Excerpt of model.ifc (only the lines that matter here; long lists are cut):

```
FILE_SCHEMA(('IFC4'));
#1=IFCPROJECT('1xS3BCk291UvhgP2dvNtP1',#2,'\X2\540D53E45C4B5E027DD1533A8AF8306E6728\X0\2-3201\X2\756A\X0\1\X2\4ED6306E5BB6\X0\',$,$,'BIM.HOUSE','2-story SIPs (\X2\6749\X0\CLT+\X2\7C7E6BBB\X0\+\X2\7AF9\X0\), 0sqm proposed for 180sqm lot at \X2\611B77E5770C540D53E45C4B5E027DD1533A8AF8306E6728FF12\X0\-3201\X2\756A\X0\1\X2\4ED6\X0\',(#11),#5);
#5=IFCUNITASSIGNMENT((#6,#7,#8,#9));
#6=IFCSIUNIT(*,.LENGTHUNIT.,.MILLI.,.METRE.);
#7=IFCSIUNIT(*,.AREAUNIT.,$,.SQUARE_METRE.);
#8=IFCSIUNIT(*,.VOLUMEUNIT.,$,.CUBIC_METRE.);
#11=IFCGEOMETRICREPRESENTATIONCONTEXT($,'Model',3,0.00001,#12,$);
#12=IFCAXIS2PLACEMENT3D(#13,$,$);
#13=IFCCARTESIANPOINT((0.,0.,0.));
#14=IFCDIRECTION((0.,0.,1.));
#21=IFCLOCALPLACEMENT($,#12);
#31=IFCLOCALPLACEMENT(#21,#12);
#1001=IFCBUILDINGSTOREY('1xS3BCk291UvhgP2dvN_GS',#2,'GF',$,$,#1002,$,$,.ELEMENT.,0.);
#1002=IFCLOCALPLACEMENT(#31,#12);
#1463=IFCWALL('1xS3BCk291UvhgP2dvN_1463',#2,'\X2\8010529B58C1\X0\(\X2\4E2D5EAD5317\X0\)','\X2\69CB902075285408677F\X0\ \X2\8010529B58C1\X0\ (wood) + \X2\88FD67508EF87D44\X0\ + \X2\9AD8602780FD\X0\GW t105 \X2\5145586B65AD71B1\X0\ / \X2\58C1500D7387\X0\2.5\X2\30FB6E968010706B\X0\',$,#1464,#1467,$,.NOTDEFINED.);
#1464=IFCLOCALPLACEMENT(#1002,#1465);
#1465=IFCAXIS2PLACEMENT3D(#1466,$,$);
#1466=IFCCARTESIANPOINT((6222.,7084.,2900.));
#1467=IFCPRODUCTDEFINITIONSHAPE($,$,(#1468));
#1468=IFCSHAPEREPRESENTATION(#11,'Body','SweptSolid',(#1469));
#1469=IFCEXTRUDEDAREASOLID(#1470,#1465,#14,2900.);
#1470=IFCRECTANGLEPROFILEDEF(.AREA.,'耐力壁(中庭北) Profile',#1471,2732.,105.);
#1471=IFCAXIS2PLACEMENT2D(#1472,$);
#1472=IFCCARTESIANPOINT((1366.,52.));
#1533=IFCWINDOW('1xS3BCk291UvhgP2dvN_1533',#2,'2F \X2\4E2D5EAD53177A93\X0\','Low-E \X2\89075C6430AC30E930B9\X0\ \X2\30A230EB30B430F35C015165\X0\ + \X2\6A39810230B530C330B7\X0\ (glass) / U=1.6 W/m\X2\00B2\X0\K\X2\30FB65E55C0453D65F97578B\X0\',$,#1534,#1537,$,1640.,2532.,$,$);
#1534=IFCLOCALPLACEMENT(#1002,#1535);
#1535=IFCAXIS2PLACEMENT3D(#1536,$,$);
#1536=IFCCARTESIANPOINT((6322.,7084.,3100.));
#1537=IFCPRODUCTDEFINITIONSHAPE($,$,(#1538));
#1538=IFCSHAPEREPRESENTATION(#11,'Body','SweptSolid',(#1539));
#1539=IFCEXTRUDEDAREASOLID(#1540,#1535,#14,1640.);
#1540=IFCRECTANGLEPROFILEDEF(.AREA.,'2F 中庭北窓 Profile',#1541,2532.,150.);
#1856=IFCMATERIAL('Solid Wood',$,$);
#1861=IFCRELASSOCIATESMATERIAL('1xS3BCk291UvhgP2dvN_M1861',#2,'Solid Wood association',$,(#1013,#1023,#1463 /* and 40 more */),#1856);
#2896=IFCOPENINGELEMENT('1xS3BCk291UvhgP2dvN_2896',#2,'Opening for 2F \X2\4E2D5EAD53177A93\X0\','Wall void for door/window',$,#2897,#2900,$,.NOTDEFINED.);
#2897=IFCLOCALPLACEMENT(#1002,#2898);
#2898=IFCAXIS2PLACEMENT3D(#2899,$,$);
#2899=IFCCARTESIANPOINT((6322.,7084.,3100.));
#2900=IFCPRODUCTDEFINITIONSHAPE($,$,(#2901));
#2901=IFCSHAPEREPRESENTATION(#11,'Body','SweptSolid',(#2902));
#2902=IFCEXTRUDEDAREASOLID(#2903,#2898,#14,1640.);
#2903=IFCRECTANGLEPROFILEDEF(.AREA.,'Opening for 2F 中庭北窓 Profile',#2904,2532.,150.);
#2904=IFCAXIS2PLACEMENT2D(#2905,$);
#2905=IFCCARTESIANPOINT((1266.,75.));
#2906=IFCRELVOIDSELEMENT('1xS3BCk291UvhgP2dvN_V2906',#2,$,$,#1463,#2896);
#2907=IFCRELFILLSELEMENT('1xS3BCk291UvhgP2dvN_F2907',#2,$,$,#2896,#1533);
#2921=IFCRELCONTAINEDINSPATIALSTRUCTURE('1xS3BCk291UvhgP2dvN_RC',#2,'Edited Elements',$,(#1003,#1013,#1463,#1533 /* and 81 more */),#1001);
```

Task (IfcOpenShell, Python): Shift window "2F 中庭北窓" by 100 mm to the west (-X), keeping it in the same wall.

```python
import ifcopenshell
import ifcopenshell.api.geometry
import ifcopenshell.util.placement
import ifcopenshell.util.unit

model = ifcopenshell.open("model.ifc")
unit_scale = ifcopenshell.util.unit.calculate_unit_scale(model)

window = model.by_id(1533)
opening = window.FillsVoids[0].RelatingOpeningElement
wall = opening.VoidsElements[0].RelatingBuildingElement

wall_matrix = ifcopenshell.util.placement.get_local_placement(wall.ObjectPlacement)
shift = wall_matrix[:3, 0] * -0.1 / unit_scale
before = ifcopenshell.util.placement.get_local_placement(window.ObjectPlacement)[:3, 3].copy()

# The window is not placed relative to its opening, so move both.
for product in (opening, window):
    matrix = ifcopenshell.util.placement.get_local_placement(product.ObjectPlacement)
    matrix[:3, 3] += shift
    ifcopenshell.api.geometry.edit_object_placement(model, product=product, matrix=matrix, is_si=False)

after = ifcopenshell.util.placement.get_local_placement(window.ObjectPlacement)[:3, 3]
print("window moved by", (after - before).round(3) + 0.0)

model.write("model_v2.ifc")
```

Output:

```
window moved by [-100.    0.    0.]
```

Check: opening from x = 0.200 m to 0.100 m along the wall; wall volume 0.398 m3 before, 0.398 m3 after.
